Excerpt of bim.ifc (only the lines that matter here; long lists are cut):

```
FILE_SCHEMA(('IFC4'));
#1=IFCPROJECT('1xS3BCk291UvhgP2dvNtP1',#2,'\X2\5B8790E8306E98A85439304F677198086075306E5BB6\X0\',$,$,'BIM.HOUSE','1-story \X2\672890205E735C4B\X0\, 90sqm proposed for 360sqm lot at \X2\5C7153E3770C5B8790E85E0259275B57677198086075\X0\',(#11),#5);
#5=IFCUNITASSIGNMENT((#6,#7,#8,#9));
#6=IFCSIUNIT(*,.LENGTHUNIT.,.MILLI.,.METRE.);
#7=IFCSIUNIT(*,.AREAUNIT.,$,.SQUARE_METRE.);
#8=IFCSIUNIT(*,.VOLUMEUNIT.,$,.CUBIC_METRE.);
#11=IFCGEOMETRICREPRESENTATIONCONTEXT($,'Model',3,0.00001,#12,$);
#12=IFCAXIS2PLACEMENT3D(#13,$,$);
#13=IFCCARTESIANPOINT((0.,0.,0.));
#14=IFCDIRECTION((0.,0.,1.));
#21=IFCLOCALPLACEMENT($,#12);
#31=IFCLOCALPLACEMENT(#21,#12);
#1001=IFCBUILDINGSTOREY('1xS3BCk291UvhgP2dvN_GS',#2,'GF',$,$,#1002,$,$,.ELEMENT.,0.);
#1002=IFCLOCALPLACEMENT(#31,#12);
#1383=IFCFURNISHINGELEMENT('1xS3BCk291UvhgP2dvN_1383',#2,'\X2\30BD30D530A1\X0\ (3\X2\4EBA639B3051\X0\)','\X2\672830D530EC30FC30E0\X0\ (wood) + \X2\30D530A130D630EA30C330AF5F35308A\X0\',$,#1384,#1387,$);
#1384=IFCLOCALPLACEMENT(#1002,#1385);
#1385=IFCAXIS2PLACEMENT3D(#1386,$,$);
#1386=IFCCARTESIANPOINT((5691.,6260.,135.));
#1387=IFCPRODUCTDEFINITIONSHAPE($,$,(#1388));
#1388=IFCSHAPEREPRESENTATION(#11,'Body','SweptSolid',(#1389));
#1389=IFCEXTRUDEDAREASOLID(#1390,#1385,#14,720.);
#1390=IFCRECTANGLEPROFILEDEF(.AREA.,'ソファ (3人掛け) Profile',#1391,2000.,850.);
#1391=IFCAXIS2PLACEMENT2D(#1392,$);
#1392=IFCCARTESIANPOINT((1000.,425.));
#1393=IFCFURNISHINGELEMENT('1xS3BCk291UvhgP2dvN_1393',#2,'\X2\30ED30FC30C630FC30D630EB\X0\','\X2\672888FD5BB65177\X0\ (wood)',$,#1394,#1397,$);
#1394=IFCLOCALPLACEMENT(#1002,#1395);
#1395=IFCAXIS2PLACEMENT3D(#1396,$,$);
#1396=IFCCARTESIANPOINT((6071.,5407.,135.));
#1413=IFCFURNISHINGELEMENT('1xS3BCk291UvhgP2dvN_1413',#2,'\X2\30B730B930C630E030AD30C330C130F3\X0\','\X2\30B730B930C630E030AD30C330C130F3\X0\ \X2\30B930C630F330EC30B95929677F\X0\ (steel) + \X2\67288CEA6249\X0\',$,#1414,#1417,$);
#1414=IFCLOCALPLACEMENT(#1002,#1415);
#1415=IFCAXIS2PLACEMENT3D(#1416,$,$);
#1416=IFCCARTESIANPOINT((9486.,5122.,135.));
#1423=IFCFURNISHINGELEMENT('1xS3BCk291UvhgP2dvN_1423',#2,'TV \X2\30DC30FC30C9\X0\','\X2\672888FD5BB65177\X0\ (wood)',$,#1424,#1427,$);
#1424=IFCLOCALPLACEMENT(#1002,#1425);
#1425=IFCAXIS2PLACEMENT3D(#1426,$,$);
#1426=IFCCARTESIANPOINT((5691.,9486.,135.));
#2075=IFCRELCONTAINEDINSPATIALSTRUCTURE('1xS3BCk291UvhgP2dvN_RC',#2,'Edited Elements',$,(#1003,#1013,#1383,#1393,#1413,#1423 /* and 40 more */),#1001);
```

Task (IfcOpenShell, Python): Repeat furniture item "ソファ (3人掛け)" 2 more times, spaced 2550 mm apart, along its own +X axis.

```python
import ifcopenshell
import ifcopenshell.api.geometry
import ifcopenshell.api.root
import ifcopenshell.util.element
import ifcopenshell.util.placement
import ifcopenshell.util.unit

model = ifcopenshell.open("bim.ifc")
unit_scale = ifcopenshell.util.unit.calculate_unit_scale(model)


def reuse_history(source, copy):
    """copy_class also copies each property set's owner history, people and application; keep the originals."""
    for rel in copy.IsDefinedBy:
        if rel.is_a("IfcRelDefinesByProperties") and (history := rel.RelatingPropertyDefinition.OwnerHistory):
            rel.RelatingPropertyDefinition.OwnerHistory = source.OwnerHistory
            ifcopenshell.util.element.remove_deep2(model, history)


source = model.by_id(1383)
base = ifcopenshell.util.placement.get_local_placement(source.ObjectPlacement)
step = base[:3, 0] * 2.55 / unit_scale

for i in range(1, 3):
    copy = ifcopenshell.api.root.copy_class(model, product=source)
    copy.Representation = ifcopenshell.util.element.copy_deep(
        model, source.Representation, exclude=["IfcGeometricRepresentationContext", "IfcRepresentationMap"]
    )
    reuse_history(source, copy)
    matrix = base.copy()
    matrix[:3, 3] += i * step
    print("added at", matrix[:3, 3].round(3) + 0.0)
    ifcopenshell.api.geometry.edit_object_placement(model, product=copy, matrix=matrix, is_si=False)

model.write("bim_updated.ifc")
```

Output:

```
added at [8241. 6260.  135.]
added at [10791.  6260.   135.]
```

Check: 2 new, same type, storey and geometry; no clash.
